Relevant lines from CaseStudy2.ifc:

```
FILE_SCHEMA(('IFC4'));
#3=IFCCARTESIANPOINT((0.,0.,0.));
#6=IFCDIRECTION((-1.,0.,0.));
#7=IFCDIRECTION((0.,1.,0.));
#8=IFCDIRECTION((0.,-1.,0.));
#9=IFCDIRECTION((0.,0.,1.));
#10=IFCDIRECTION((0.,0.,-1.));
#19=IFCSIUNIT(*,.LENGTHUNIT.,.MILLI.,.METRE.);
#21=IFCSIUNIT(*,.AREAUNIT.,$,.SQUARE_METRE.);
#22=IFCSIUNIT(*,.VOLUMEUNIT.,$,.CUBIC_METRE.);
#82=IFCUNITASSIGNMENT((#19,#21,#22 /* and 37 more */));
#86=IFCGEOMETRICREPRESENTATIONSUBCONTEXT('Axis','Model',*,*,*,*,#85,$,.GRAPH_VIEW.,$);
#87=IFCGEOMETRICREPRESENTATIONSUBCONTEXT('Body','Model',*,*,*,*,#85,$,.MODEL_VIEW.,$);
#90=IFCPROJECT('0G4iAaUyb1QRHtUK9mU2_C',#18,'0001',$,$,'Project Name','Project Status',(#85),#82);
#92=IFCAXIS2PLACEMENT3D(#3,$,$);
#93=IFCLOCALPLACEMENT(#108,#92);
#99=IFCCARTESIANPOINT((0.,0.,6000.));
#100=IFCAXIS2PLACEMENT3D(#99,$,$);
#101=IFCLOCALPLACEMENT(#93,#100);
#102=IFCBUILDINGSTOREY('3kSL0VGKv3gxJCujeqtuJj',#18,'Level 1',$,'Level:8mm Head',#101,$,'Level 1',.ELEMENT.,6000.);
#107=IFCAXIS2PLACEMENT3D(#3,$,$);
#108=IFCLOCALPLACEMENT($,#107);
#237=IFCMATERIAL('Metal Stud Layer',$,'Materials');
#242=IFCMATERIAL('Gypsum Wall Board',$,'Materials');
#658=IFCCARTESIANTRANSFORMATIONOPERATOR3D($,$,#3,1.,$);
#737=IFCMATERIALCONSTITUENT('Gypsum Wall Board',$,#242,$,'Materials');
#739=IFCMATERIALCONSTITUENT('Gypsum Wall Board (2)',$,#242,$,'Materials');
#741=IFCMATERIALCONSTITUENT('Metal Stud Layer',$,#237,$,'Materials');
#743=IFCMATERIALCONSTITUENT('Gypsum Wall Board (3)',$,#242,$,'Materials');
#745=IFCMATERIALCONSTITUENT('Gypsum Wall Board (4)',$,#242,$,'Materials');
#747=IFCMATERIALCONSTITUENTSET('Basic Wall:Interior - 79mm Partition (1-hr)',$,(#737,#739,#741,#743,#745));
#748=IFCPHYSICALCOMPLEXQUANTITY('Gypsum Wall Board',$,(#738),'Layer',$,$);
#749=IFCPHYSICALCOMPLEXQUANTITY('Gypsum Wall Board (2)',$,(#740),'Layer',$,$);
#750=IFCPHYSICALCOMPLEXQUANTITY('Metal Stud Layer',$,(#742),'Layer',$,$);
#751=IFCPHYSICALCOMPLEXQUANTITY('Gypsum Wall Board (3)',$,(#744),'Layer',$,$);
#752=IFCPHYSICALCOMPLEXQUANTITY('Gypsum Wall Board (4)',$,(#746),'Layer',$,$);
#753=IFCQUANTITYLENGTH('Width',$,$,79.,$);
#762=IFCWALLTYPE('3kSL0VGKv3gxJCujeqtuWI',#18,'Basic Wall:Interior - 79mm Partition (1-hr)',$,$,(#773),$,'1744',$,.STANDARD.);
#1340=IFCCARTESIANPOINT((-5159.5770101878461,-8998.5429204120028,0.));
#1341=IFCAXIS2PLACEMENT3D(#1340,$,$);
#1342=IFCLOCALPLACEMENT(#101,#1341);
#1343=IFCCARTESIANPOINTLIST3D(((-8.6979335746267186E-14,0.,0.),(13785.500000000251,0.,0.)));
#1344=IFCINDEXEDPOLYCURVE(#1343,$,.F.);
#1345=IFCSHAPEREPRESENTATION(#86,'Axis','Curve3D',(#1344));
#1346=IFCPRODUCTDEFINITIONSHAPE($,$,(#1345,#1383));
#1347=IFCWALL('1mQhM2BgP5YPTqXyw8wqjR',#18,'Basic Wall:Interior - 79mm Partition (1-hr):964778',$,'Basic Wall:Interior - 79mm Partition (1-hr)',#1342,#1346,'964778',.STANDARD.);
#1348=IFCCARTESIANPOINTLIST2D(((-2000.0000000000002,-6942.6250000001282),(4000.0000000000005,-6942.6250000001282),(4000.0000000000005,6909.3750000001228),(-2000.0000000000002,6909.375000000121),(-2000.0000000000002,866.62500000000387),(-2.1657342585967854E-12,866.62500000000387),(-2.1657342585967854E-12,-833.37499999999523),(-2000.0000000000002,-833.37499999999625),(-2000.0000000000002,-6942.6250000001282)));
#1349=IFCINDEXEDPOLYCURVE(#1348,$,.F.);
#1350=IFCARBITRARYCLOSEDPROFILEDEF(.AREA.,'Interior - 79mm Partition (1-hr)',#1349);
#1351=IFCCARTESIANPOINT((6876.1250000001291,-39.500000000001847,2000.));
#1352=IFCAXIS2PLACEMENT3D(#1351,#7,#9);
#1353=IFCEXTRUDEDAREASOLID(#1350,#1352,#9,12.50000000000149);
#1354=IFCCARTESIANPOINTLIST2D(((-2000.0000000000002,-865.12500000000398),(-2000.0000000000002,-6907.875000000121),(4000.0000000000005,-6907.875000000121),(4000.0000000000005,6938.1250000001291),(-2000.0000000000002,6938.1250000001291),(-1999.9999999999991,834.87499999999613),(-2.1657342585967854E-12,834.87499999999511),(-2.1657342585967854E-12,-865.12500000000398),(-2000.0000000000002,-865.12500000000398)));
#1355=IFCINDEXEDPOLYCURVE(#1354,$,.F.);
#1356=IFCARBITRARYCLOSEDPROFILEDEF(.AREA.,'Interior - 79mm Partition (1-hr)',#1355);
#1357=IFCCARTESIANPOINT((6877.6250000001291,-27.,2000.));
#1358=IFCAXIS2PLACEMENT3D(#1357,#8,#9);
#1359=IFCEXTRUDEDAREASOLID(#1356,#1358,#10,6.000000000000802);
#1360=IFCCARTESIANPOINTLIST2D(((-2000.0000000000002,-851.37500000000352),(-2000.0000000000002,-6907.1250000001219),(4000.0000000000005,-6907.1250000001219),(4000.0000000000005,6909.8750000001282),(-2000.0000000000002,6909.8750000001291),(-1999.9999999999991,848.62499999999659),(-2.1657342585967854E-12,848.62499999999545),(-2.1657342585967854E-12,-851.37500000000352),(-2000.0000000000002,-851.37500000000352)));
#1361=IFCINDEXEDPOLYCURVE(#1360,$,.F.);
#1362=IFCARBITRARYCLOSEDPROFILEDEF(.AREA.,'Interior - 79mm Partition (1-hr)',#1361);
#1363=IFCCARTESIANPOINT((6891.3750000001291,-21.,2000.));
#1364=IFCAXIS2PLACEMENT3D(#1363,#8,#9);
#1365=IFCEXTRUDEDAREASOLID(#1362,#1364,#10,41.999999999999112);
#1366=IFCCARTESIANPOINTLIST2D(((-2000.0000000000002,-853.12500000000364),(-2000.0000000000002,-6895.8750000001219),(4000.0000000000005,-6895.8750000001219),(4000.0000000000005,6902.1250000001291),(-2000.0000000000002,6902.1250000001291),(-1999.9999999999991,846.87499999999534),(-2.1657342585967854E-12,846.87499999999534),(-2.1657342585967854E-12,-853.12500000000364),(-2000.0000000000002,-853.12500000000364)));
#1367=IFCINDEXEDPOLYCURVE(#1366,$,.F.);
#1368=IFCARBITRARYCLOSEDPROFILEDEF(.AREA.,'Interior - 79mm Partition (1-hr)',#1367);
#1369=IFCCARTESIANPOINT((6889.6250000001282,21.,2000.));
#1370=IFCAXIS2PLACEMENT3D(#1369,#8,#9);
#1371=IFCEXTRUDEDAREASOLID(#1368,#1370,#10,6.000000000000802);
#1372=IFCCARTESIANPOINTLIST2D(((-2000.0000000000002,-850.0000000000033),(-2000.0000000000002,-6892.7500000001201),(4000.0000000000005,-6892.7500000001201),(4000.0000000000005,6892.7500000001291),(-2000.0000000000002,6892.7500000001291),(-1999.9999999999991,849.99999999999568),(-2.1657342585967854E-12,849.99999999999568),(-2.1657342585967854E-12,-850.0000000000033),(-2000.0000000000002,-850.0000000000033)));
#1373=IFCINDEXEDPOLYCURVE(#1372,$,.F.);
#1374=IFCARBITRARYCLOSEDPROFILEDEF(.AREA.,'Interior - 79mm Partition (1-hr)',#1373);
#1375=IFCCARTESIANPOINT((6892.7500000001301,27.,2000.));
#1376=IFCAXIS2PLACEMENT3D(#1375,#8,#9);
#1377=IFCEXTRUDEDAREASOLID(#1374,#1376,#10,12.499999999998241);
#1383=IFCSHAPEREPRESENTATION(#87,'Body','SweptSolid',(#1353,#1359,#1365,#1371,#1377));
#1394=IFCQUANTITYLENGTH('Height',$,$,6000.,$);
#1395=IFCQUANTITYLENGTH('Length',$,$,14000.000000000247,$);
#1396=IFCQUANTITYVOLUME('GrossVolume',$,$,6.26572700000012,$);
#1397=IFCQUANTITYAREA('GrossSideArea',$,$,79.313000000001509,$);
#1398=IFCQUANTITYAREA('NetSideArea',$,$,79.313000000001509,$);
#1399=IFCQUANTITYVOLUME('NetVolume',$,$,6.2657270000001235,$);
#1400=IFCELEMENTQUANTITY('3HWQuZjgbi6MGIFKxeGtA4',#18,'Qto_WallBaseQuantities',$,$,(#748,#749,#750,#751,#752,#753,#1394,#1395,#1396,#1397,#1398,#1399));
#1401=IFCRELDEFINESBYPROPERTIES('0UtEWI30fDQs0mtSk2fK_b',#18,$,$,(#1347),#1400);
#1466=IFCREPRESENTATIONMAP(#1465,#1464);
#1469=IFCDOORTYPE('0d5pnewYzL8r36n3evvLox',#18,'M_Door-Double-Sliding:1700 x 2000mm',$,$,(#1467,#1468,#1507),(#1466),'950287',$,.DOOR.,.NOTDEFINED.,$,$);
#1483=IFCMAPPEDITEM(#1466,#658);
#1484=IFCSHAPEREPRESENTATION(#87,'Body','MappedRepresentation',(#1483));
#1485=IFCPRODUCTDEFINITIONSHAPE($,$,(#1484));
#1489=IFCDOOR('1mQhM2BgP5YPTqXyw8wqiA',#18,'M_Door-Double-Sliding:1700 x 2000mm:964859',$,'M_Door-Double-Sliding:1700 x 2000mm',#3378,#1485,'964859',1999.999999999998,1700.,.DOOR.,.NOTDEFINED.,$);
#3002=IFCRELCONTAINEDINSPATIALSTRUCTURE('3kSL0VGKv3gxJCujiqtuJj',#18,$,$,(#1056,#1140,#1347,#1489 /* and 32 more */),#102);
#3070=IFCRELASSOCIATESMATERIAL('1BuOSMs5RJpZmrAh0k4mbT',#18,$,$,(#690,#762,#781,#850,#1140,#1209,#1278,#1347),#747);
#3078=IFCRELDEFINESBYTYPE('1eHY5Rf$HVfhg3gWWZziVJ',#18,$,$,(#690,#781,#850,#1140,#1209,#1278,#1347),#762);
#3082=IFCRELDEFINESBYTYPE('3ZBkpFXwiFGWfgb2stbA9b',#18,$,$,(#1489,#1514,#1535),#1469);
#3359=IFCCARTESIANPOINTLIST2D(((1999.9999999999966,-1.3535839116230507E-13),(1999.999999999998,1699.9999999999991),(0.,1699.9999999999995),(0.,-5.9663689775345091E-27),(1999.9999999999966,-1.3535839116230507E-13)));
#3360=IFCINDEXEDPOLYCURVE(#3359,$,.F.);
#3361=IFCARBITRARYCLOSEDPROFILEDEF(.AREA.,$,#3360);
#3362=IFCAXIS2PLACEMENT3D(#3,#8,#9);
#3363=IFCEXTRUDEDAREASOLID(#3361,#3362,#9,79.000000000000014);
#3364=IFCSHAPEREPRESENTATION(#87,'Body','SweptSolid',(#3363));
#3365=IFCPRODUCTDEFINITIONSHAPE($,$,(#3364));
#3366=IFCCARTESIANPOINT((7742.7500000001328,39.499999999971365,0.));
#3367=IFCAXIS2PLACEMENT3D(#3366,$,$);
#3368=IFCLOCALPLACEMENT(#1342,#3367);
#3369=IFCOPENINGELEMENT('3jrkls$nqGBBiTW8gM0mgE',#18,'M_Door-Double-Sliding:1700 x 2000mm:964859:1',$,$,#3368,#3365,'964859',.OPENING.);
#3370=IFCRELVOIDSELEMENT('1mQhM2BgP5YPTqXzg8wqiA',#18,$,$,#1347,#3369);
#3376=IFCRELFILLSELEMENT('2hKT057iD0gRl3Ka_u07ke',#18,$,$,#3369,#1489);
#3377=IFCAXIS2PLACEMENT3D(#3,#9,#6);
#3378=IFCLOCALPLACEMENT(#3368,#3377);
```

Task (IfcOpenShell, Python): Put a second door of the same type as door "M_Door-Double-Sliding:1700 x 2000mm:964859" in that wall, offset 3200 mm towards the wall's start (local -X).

```python
import ifcopenshell
import ifcopenshell.api.feature
import ifcopenshell.api.geometry
import ifcopenshell.api.pset
import ifcopenshell.api.root
import ifcopenshell.geom
import ifcopenshell.util.element
import ifcopenshell.util.placement
import ifcopenshell.util.shape
import ifcopenshell.util.unit

model = ifcopenshell.open("CaseStudy2.ifc")
area_scale = ifcopenshell.util.unit.calculate_unit_scale(model, "AREAUNIT")
volume_scale = ifcopenshell.util.unit.calculate_unit_scale(model, "VOLUMEUNIT")
settings = ifcopenshell.geom.settings()


def volume(element):
    """Net volume in cubic metres, openings subtracted."""
    shape = ifcopenshell.geom.create_shape(settings, element)
    return ifcopenshell.util.shape.get_volume(shape.geometry)


def reuse_history(source, copy):
    """copy_class also copies each property set's owner history, people and application; keep the originals."""
    for rel in copy.IsDefinedBy:
        if rel.is_a("IfcRelDefinesByProperties") and (history := rel.RelatingPropertyDefinition.OwnerHistory):
            rel.RelatingPropertyDefinition.OwnerHistory = source.OwnerHistory
            ifcopenshell.util.element.remove_deep2(model, history)


door = model.by_guid("1mQhM2BgP5YPTqXyw8wqiA")
opening = door.FillsVoids[0].RelatingOpeningElement
wall = opening.VoidsElements[0].RelatingBuildingElement
before = volume(wall)
shift = ifcopenshell.util.placement.get_local_placement(wall.ObjectPlacement)[:3, 0] * -3200.0

# copy_class copies the void relationship, type, container and properties, but no geometry.
new_opening = ifcopenshell.api.root.copy_class(model, product=opening)
new_opening.Representation = ifcopenshell.util.element.copy_deep(
    model, opening.Representation, exclude=["IfcGeometricRepresentationContext", "IfcRepresentationMap"]
)
new_opening.Name = "M_Door-Double-Sliding:1700 x 2000mm"
new_opening.Tag = None
reuse_history(opening, new_opening)
new_door = ifcopenshell.api.root.copy_class(model, product=door)
new_door.Representation = ifcopenshell.util.element.copy_deep(
    model, door.Representation, exclude=["IfcGeometricRepresentationContext", "IfcRepresentationMap"]
)
new_door.Name = "M_Door-Double-Sliding:1700 x 2000mm"
new_door.Tag = None
reuse_history(door, new_door)
ifcopenshell.api.feature.add_filling(model, opening=new_opening, element=new_door)

for old, new in ((opening, new_opening), (door, new_door)):
    matrix = ifcopenshell.util.placement.get_local_placement(old.ObjectPlacement)
    matrix[:3, 3] += shift
    ifcopenshell.api.geometry.edit_object_placement(model, product=new, matrix=matrix, is_si=False)

after = volume(wall)
thickness = 0.079  # wall thickness in metres

# Update the wall's stored quantities.
qto = model.by_id(ifcopenshell.util.element.get_pset(wall, "Qto_WallBaseQuantities", should_inherit=False)["id"])
ifcopenshell.api.pset.edit_qto(model, qto=qto, properties={
    "NetSideArea": after / thickness / area_scale,
    "NetVolume": after / volume_scale,
})

print(f"wall volume {before:.3f} -> {after:.3f} m3")

model.write("CaseStudy2-out.ifc")
```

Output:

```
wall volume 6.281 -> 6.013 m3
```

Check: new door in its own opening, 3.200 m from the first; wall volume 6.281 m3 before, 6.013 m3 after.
